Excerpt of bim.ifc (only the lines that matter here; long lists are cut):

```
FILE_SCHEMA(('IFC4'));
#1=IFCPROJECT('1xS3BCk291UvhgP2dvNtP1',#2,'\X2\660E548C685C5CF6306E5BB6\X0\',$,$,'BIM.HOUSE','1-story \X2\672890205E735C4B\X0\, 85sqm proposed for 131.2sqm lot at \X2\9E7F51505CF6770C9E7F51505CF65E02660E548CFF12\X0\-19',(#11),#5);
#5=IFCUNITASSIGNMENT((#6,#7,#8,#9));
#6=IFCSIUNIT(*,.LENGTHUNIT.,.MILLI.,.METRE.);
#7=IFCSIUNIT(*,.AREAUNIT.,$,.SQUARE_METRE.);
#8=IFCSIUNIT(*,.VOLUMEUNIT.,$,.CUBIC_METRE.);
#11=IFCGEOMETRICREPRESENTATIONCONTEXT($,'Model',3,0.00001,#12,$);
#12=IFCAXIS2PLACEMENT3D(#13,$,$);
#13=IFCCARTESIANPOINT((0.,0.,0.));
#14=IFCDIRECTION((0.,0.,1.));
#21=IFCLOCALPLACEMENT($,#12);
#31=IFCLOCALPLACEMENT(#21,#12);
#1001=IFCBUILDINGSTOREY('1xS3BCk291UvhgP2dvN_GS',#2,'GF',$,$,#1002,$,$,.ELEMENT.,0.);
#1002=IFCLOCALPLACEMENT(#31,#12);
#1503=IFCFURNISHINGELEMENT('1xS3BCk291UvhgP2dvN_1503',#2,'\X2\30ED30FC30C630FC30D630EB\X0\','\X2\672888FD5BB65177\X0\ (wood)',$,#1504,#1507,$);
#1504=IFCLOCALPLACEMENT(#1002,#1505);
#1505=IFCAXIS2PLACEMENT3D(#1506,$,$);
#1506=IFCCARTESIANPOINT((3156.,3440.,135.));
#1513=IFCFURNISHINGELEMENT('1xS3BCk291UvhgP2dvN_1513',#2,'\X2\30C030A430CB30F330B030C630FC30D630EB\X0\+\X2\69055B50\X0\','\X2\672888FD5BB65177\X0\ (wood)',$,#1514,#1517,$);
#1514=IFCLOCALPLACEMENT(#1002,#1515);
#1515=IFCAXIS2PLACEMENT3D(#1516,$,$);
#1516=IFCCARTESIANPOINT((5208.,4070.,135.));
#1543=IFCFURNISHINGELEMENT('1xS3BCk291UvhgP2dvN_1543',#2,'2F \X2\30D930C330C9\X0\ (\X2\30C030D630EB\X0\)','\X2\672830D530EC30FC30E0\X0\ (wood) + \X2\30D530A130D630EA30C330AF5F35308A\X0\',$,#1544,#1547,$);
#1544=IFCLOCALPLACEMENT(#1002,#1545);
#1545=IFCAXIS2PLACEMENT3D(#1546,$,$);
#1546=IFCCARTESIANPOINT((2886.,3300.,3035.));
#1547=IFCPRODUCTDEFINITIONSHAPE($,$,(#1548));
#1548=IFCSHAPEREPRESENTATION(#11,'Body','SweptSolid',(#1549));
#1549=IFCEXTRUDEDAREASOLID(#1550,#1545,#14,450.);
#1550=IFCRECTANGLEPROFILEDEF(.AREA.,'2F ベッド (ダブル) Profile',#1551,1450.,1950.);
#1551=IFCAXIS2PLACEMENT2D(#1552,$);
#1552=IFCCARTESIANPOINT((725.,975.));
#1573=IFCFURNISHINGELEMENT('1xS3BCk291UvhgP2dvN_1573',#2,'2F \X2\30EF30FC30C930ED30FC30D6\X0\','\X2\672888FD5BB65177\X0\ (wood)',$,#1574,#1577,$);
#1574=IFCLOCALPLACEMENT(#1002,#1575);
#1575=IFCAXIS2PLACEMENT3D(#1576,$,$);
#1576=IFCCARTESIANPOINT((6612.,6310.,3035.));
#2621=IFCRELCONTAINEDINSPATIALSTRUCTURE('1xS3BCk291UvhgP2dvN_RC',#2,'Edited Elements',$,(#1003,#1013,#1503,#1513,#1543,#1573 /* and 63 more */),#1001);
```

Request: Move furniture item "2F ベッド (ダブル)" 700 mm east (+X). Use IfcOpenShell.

```python
import ifcopenshell
import ifcopenshell.api.geometry
import ifcopenshell.util.placement
import ifcopenshell.util.unit

model = ifcopenshell.open("bim.ifc")
unit_scale = ifcopenshell.util.unit.calculate_unit_scale(model)

item = model.by_guid("1xS3BCk291UvhgP2dvN_1543")
matrix = ifcopenshell.util.placement.get_local_placement(item.ObjectPlacement)
matrix[0, 3] += 0.7 / unit_scale
ifcopenshell.api.geometry.edit_object_placement(model, product=item, matrix=matrix, is_si=False)

print(ifcopenshell.util.placement.get_local_placement(item.ObjectPlacement).round(3) + 0.0)

model.write("bim_edited.ifc")
```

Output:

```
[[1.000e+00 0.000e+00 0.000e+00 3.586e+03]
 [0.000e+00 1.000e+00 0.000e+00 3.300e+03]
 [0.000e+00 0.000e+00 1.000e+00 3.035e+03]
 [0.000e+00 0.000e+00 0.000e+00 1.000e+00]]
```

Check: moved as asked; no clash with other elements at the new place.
